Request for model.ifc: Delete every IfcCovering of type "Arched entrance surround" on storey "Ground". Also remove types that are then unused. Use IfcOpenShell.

First a look at what the model holds.

```python
import ifcopenshell
import ifcopenshell.util.element

model = ifcopenshell.open("model.ifc")
print(model.schema)
storey = next(s for s in model.by_type("IfcBuildingStorey") if s.Name == "Ground")
coverings = [e for e in ifcopenshell.util.element.get_decomposition(storey) if e.is_a("IfcCovering")]
seen = {}
for e in coverings:
    element_type = ifcopenshell.util.element.get_type(e)
    name = element_type.Name if element_type not in (None, e) else None
    seen[name] = seen.get(name, 0) + 1
for name, count in sorted(seen.items(), key=str):
    print(count, "x", name)
```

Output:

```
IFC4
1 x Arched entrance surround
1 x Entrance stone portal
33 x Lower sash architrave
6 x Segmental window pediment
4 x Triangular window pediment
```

```python
import ifcopenshell
import ifcopenshell.api.root
import ifcopenshell.util.element

model = ifcopenshell.open("model.ifc")

storey = next(s for s in model.by_type("IfcBuildingStorey") if s.Name == "Ground")
coverings = [e for e in ifcopenshell.util.element.get_decomposition(storey) if e.is_a("IfcCovering")]
targets = [e for e in coverings if (t := ifcopenshell.util.element.get_type(e)) not in (None, e) and t.Name == "Arched entrance surround"]
types = {ifcopenshell.util.element.get_type(e) for e in targets} - {None, *targets}

for e in targets:
    ifcopenshell.api.root.remove_product(model, product=e)
print(len(targets), "removed")

unused = [t for t in types if not ifcopenshell.util.element.get_types(t)]
for t in unused:
    ifcopenshell.api.root.remove_product(model, product=t)
print(len(unused), "unused types removed")

model.write("model_edited.ifc")
```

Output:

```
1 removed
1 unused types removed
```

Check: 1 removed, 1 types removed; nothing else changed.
